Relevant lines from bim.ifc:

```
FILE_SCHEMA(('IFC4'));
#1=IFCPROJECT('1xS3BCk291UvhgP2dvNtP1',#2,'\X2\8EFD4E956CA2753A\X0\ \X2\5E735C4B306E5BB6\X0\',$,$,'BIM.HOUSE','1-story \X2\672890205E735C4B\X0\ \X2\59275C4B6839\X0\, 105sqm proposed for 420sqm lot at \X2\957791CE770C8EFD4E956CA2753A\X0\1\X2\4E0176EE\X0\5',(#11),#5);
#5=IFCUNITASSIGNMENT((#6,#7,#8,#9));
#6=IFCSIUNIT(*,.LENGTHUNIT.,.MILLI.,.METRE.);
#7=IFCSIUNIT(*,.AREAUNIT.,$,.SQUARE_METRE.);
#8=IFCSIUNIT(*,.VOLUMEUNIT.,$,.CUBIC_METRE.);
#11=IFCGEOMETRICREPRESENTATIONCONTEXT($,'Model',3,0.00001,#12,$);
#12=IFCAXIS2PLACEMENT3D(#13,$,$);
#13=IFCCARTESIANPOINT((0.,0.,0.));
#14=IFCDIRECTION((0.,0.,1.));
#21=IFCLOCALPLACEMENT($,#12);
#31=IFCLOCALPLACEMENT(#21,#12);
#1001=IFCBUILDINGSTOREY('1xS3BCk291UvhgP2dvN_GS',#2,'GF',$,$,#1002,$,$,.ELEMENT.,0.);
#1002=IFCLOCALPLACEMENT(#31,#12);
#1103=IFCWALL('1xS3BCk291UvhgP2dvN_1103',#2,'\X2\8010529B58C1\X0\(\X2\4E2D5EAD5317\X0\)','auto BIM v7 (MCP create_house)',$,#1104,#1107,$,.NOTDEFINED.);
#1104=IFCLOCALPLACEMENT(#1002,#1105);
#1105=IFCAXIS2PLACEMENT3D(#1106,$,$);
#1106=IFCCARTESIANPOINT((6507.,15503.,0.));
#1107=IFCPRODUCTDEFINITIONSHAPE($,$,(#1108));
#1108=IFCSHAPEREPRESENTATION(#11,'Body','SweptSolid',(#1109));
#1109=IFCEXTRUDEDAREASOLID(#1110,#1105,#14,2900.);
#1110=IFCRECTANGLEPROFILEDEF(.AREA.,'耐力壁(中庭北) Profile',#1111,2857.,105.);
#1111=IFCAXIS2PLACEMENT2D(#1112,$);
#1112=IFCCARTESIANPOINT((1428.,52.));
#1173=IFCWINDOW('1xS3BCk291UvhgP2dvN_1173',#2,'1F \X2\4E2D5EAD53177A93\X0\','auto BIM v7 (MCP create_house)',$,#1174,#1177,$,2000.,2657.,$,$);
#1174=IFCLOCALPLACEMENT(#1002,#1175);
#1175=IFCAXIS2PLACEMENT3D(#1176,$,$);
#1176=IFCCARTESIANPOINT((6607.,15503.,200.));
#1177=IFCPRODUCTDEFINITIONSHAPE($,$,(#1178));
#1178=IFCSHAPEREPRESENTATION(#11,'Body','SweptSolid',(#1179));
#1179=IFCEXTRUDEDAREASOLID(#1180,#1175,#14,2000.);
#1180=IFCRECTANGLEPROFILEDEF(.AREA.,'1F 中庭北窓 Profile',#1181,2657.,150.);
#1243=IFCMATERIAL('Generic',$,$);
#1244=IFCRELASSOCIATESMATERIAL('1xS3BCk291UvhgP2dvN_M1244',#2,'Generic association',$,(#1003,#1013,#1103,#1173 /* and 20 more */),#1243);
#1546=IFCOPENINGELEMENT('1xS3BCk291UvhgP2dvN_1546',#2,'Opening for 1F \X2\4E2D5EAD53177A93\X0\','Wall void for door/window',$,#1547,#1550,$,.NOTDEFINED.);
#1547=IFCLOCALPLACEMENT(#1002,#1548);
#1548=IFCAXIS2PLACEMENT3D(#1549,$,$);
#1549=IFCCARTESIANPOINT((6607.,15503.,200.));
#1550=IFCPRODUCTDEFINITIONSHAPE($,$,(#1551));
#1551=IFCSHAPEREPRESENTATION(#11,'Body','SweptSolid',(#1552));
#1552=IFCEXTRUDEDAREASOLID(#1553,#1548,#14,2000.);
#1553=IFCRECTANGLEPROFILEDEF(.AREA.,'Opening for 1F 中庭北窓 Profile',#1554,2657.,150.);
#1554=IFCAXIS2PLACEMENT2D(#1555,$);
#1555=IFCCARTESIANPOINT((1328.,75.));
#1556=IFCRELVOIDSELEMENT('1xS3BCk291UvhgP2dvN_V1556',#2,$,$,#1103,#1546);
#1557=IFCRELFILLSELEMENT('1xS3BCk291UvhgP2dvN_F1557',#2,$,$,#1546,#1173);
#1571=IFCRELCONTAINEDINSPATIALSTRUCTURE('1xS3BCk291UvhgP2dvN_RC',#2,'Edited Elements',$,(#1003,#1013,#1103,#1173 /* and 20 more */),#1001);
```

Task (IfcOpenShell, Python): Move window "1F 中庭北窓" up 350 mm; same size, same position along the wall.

```python
import numpy as np
import ifcopenshell
import ifcopenshell.api.geometry
import ifcopenshell.util.placement
import ifcopenshell.util.unit

model = ifcopenshell.open("bim.ifc")
unit_scale = ifcopenshell.util.unit.calculate_unit_scale(model)

window = model.by_guid("1xS3BCk291UvhgP2dvN_1173")
opening = window.FillsVoids[0].RelatingOpeningElement
dz = 350.0

shift = np.array([0.0, 0.0, dz])
# The window is not placed relative to its opening, so move both.
for product in (opening, window):
    matrix = ifcopenshell.util.placement.get_local_placement(product.ObjectPlacement)
    matrix[:3, 3] += shift
    ifcopenshell.api.geometry.edit_object_placement(model, product=product, matrix=matrix, is_si=False)

print(f"moved by {dz * unit_scale:+.3f} m")

model.write("bim_v2.ifc")
```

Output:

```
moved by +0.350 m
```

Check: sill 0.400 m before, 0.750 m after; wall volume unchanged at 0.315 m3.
